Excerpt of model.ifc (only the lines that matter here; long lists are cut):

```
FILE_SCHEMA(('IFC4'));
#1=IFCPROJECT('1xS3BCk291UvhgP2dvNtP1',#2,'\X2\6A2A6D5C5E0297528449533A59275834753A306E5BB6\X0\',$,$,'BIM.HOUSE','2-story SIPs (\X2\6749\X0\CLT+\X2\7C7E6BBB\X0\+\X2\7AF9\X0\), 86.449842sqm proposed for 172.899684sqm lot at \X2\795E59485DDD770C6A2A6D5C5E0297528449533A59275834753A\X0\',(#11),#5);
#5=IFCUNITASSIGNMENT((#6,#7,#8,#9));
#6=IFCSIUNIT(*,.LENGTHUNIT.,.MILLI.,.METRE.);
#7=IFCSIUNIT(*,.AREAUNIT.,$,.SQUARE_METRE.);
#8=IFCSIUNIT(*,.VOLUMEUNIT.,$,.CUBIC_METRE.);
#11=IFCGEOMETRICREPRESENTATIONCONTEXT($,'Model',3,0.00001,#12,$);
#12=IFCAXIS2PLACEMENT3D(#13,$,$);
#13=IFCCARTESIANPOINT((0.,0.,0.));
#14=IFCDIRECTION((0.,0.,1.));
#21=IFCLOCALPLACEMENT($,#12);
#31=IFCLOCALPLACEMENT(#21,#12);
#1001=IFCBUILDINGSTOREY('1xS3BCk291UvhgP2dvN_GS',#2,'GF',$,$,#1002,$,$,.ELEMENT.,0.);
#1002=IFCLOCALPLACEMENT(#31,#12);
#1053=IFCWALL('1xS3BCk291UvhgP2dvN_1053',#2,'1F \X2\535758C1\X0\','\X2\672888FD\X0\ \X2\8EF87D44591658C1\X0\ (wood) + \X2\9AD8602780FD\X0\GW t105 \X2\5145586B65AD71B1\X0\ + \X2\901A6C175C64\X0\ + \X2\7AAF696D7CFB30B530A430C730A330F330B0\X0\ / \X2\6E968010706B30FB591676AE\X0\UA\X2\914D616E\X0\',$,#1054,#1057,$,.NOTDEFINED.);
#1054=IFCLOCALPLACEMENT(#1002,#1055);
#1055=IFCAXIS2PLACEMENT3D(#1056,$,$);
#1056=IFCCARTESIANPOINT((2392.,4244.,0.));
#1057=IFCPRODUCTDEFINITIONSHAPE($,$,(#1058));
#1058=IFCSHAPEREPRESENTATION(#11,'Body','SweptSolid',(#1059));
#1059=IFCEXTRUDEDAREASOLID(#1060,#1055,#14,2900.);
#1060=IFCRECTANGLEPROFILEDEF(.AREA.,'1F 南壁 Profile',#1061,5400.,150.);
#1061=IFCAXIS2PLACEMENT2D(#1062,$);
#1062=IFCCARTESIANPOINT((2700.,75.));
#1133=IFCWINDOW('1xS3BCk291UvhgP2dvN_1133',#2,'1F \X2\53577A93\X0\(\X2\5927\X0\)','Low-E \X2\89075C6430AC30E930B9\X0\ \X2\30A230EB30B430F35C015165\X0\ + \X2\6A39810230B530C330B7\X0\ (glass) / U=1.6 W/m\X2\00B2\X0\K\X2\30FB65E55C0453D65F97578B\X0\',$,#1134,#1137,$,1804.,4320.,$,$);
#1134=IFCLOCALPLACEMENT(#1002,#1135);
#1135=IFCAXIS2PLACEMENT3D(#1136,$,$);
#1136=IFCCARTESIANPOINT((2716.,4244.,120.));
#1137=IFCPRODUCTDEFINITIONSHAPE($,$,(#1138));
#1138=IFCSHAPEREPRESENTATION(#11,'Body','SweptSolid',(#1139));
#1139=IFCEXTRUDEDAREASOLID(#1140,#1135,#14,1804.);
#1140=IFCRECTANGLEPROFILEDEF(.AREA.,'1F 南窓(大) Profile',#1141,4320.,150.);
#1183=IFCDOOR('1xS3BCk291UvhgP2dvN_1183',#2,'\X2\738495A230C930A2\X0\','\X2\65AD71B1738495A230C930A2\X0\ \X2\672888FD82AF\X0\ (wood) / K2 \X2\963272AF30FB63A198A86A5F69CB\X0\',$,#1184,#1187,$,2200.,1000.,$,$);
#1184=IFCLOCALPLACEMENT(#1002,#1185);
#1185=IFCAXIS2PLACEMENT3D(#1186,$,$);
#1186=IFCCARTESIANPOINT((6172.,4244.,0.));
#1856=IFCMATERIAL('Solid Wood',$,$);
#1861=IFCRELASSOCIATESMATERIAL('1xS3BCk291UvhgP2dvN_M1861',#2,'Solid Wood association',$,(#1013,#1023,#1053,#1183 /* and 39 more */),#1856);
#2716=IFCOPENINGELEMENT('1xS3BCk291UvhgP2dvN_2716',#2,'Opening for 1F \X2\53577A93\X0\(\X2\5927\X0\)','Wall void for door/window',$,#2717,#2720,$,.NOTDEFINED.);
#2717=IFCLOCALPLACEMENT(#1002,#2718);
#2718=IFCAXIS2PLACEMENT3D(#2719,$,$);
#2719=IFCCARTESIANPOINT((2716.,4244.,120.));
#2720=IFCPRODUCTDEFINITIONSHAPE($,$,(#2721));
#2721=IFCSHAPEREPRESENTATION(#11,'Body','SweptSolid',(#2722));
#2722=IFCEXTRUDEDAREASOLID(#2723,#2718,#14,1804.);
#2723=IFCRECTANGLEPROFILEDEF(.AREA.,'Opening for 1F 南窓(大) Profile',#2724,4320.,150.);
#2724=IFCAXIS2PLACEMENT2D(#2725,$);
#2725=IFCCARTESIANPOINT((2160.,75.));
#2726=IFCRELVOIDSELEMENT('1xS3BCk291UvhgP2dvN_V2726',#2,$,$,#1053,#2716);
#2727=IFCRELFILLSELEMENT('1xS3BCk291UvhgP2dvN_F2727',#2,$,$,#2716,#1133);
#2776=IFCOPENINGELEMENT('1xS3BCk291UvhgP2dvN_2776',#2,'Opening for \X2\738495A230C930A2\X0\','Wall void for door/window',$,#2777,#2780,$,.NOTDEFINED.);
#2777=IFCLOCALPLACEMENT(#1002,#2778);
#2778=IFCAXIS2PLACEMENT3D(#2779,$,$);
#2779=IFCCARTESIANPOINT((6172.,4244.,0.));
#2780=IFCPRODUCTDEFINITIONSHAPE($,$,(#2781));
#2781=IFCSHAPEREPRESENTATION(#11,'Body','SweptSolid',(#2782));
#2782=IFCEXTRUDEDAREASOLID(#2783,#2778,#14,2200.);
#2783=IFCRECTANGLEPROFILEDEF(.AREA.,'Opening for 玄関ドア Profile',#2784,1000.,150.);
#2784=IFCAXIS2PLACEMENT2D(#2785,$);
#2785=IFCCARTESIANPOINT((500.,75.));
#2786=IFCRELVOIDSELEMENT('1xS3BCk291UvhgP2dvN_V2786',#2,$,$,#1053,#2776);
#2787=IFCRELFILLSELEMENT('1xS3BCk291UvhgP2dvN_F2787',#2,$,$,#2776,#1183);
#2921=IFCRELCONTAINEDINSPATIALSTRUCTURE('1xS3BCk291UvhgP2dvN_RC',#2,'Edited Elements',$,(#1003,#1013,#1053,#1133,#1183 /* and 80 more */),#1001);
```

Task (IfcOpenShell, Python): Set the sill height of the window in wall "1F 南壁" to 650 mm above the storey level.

```python
import numpy as np
import ifcopenshell
import ifcopenshell.api.geometry
import ifcopenshell.geom
import ifcopenshell.util.element
import ifcopenshell.util.placement
import ifcopenshell.util.shape
import ifcopenshell.util.unit

model = ifcopenshell.open("model.ifc")
unit_scale = ifcopenshell.util.unit.calculate_unit_scale(model)

window = model.by_id(1133)
opening = window.FillsVoids[0].RelatingOpeningElement
storey = ifcopenshell.util.element.get_container(window, ifc_class="IfcBuildingStorey")
level = ifcopenshell.util.placement.get_local_placement(storey.ObjectPlacement)[2, 3]

# The opening's origin need not be at the sill, so measure its lowest point.
shape = ifcopenshell.geom.create_shape(ifcopenshell.geom.settings(), opening)
bottom = ifcopenshell.util.shape.get_shape_bottom_elevation(shape, shape.geometry) / unit_scale
dz = level + 0.65 / unit_scale - bottom

shift = np.array([0.0, 0.0, dz])
# The window is not placed relative to its opening, so move both.
for product in (opening, window):
    matrix = ifcopenshell.util.placement.get_local_placement(product.ObjectPlacement)
    matrix[:3, 3] += shift
    ifcopenshell.api.geometry.edit_object_placement(model, product=product, matrix=matrix, is_si=False)

print(f"moved by {dz * unit_scale:+.3f} m")

model.write("model_updated.ifc")
```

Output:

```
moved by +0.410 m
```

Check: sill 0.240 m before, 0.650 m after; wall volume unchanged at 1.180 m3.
